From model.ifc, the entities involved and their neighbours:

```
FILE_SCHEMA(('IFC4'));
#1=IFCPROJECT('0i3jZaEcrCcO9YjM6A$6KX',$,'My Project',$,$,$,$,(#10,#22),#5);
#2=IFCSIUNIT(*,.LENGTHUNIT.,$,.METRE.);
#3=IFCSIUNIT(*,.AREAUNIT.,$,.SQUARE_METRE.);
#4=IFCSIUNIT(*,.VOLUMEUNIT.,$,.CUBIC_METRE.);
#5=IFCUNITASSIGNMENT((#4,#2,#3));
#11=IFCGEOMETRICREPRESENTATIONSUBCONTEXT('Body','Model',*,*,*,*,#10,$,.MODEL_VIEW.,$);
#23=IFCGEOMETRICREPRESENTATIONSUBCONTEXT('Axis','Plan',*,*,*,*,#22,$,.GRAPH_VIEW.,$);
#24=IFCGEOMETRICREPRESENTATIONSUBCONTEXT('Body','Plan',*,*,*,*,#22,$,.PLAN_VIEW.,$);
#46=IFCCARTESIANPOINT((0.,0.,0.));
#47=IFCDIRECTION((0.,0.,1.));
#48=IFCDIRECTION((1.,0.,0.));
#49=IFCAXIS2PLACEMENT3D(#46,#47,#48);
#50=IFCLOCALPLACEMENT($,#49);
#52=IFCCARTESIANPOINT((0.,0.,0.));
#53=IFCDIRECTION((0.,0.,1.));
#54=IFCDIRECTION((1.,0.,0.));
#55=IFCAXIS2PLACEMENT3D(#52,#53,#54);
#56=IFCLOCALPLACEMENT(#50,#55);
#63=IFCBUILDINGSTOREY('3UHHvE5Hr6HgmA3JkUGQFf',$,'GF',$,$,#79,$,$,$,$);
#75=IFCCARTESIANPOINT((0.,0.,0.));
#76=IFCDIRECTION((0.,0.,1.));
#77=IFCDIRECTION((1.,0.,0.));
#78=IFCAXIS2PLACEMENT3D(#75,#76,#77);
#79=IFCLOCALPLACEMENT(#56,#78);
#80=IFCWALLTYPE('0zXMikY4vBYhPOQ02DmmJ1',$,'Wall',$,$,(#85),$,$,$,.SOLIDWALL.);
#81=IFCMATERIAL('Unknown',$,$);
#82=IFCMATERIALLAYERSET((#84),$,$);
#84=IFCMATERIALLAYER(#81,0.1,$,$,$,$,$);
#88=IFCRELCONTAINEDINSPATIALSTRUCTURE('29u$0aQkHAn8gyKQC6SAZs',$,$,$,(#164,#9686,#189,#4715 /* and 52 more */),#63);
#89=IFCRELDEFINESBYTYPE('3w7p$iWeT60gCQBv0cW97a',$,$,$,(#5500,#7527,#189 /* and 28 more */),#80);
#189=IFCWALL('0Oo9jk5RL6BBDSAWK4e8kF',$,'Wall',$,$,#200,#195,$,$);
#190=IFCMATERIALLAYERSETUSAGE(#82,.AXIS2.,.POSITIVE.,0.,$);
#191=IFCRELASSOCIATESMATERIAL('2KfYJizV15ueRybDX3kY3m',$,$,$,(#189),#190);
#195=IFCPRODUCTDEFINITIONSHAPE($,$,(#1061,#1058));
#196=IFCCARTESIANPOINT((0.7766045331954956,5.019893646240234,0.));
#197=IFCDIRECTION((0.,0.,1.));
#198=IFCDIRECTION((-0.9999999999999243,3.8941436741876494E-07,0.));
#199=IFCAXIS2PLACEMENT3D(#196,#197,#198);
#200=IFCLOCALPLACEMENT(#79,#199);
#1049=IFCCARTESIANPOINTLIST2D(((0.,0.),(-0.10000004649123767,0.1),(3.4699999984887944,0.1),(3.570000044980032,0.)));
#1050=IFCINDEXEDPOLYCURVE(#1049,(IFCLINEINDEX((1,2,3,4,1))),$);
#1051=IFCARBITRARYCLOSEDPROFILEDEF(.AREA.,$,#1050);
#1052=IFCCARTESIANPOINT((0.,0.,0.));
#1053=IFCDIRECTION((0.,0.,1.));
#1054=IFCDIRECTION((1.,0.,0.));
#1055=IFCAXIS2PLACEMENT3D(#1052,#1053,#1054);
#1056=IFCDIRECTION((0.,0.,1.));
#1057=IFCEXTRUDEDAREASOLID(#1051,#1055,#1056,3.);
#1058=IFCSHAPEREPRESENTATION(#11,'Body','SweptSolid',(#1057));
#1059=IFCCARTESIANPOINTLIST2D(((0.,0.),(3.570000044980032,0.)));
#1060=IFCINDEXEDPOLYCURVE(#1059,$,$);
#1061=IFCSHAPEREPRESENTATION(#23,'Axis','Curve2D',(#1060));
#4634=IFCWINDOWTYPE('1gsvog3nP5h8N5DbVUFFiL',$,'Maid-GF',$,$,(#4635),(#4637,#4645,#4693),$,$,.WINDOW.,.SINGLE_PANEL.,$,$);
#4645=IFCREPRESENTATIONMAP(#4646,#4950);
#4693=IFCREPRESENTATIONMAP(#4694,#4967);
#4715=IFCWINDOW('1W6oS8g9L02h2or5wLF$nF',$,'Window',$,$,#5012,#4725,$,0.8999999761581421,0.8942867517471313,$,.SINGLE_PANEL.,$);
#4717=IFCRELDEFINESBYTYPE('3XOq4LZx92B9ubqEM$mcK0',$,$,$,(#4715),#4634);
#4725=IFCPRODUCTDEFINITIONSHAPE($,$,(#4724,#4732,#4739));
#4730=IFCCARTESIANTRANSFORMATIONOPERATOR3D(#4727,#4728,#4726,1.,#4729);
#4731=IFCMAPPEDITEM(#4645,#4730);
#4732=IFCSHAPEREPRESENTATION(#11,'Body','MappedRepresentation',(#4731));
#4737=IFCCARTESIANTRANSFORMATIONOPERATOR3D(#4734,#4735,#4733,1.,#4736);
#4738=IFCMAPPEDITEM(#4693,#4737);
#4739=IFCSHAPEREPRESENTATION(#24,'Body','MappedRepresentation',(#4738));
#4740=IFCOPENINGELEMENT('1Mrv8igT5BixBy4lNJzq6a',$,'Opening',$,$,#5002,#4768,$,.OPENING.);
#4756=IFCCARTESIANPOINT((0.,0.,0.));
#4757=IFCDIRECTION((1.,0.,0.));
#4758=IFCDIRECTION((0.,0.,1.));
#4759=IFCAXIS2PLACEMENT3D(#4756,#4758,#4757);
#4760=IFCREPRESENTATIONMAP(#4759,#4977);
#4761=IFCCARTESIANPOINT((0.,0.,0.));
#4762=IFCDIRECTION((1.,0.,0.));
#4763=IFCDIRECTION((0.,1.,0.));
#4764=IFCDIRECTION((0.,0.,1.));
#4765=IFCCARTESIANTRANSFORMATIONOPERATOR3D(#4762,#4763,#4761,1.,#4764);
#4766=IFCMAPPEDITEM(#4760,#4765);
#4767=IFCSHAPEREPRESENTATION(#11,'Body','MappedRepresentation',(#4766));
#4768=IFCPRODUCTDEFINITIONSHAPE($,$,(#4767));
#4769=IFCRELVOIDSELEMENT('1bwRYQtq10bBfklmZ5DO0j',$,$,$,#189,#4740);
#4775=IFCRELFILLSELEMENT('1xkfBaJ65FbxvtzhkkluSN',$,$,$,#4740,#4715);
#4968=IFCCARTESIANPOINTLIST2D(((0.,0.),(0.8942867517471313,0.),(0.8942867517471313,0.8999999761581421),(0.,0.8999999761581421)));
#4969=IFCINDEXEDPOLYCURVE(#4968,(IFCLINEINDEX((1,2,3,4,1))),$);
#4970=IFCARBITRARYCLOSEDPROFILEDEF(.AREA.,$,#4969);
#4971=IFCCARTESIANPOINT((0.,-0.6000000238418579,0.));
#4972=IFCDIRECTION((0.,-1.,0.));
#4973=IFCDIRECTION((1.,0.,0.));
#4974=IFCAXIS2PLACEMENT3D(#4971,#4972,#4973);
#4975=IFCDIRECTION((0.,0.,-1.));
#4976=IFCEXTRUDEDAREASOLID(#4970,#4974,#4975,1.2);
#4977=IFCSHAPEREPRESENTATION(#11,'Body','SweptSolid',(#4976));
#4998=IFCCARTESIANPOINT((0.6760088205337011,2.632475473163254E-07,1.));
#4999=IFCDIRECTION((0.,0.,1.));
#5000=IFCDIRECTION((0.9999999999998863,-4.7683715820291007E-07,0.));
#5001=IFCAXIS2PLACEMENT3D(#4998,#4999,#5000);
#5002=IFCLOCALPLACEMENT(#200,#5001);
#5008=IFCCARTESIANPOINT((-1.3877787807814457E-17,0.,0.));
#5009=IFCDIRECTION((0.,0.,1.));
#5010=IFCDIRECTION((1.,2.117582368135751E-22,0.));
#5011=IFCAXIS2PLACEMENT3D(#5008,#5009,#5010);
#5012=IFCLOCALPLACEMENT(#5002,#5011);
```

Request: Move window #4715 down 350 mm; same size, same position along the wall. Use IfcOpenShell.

```python
import numpy as np
import ifcopenshell
import ifcopenshell.api.geometry
import ifcopenshell.util.placement
import ifcopenshell.util.unit

model = ifcopenshell.open("model.ifc")
unit_scale = ifcopenshell.util.unit.calculate_unit_scale(model)

window = model.by_guid("1W6oS8g9L02h2or5wLF$nF")
opening = window.FillsVoids[0].RelatingOpeningElement
dz = -0.35 / unit_scale

shift = np.array([0.0, 0.0, dz])
# The window is placed relative to its opening, so it follows when the opening moves.
matrix = ifcopenshell.util.placement.get_local_placement(opening.ObjectPlacement)
matrix[:3, 3] += shift
ifcopenshell.api.geometry.edit_object_placement(
    model, product=opening, matrix=matrix, is_si=False, should_transform_children=True
)

print(f"moved by {dz * unit_scale:+.3f} m")

model.write("model_updated.ifc")
```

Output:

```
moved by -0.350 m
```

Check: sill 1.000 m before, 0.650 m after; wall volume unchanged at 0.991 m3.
